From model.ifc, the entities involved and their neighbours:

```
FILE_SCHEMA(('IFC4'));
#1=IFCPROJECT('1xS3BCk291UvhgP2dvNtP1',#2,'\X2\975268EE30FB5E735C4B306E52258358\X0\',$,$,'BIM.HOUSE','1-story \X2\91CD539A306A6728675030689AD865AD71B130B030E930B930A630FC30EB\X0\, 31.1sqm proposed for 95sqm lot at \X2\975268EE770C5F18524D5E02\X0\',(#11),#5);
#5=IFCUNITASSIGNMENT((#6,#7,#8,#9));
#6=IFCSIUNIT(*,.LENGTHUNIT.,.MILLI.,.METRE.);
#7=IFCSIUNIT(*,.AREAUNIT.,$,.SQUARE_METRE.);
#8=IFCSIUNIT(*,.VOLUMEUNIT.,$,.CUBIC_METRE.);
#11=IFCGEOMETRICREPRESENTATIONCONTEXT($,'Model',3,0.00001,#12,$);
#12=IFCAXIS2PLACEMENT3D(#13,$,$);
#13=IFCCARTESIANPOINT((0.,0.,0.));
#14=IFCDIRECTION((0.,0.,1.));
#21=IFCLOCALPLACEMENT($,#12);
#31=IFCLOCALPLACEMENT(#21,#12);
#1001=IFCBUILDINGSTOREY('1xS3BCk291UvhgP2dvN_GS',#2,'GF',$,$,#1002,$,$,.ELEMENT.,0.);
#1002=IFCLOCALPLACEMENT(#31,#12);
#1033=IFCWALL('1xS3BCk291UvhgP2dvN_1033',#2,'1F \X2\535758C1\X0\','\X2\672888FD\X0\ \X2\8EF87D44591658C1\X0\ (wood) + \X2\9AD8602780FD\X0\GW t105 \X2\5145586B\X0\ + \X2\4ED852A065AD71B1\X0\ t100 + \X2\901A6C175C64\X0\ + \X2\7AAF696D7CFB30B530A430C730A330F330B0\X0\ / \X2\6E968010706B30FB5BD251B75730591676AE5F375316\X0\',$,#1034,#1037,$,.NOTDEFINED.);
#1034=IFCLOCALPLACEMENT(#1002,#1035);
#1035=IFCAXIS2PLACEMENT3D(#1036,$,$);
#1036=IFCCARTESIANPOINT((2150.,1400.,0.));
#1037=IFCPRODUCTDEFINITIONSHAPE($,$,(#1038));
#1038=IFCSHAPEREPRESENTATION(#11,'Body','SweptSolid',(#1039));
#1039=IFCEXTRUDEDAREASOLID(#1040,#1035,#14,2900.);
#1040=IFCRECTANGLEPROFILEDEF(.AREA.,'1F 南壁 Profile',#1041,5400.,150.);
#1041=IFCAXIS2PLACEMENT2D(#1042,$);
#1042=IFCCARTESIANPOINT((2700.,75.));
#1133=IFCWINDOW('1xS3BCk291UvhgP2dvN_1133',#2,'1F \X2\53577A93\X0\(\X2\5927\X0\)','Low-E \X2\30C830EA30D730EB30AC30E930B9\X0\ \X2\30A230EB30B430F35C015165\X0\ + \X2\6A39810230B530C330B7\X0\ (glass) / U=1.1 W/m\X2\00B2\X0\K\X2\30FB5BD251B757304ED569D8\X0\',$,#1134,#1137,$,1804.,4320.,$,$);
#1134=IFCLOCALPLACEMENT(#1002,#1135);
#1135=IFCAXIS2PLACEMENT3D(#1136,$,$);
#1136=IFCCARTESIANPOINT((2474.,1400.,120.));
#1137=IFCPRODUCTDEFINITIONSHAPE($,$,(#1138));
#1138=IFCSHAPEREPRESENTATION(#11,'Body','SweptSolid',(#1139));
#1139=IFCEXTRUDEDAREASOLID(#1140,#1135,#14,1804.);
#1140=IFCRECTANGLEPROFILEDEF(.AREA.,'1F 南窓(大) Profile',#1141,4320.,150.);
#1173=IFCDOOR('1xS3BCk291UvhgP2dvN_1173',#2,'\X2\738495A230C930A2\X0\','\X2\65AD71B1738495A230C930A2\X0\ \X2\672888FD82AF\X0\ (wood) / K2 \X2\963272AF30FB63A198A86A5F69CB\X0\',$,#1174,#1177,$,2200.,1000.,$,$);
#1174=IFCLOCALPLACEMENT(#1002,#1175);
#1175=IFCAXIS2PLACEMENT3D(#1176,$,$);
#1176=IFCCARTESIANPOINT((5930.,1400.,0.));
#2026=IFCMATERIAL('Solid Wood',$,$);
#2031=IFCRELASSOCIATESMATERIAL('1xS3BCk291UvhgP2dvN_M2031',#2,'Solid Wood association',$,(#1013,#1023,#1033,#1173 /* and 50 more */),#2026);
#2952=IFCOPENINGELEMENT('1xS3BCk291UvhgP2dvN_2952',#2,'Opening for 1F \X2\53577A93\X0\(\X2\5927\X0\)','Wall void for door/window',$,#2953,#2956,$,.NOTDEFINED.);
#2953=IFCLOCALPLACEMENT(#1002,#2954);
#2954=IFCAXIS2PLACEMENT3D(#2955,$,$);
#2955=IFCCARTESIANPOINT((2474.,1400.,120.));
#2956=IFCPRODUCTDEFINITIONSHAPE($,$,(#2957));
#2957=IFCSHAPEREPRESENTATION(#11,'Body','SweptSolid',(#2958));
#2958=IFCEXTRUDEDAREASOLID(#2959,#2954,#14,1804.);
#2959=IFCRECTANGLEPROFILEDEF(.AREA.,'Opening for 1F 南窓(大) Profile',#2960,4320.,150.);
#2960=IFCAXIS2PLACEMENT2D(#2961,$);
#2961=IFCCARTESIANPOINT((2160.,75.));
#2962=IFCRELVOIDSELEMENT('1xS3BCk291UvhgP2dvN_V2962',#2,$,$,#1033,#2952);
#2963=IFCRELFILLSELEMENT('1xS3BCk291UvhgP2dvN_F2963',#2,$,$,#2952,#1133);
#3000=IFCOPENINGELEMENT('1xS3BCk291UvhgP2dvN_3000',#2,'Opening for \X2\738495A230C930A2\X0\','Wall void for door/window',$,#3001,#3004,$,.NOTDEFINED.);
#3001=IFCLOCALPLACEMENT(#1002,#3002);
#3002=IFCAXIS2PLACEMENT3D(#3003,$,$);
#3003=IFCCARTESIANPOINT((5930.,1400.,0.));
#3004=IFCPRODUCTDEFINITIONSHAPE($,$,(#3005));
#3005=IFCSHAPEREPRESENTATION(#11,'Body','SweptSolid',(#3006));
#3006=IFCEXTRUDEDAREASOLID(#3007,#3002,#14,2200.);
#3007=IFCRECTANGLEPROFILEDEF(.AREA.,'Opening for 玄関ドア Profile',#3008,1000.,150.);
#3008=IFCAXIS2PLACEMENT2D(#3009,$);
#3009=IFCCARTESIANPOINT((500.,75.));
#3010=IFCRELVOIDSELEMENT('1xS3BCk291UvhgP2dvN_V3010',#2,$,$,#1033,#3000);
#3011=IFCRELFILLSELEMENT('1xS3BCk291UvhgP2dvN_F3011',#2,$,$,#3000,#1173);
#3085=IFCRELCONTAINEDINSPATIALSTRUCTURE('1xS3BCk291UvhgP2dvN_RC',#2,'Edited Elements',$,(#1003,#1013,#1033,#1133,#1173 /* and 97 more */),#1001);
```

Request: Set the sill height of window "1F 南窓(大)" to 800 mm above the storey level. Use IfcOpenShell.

```python
import numpy as np
import ifcopenshell
import ifcopenshell.api.geometry
import ifcopenshell.geom
import ifcopenshell.util.element
import ifcopenshell.util.placement
import ifcopenshell.util.shape
import ifcopenshell.util.unit

model = ifcopenshell.open("model.ifc")
unit_scale = ifcopenshell.util.unit.calculate_unit_scale(model)

window = model.by_guid("1xS3BCk291UvhgP2dvN_1133")
opening = window.FillsVoids[0].RelatingOpeningElement
storey = ifcopenshell.util.element.get_container(window, ifc_class="IfcBuildingStorey")
level = ifcopenshell.util.placement.get_local_placement(storey.ObjectPlacement)[2, 3]

# The opening's origin need not be at the sill, so measure its lowest point.
shape = ifcopenshell.geom.create_shape(ifcopenshell.geom.settings(), opening)
bottom = ifcopenshell.util.shape.get_shape_bottom_elevation(shape, shape.geometry) / unit_scale
dz = level + 0.8 / unit_scale - bottom

shift = np.array([0.0, 0.0, dz])
# The window is not placed relative to its opening, so move both.
for product in (opening, window):
    matrix = ifcopenshell.util.placement.get_local_placement(product.ObjectPlacement)
    matrix[:3, 3] += shift
    ifcopenshell.api.geometry.edit_object_placement(model, product=product, matrix=matrix, is_si=False)

print(f"moved by {dz * unit_scale:+.3f} m")

model.write("model_v2.ifc")
```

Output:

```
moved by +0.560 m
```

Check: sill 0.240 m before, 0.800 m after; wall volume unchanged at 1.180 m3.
